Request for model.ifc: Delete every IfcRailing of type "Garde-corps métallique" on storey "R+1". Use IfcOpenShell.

First a look at what the model holds.

```python
import ifcopenshell
import ifcopenshell.util.element

model = ifcopenshell.open("model.ifc")
print(model.schema)
storey = next(s for s in model.by_type("IfcBuildingStorey") if s.Name == "R+1")
railings = [e for e in ifcopenshell.util.element.get_decomposition(storey) if e.is_a("IfcRailing")]
seen = {}
for e in railings:
    element_type = ifcopenshell.util.element.get_type(e)
    name = element_type.Name if element_type not in (None, e) else None
    seen[name] = seen.get(name, 0) + 1
for name, count in sorted(seen.items(), key=str):
    print(count, "x", name)
```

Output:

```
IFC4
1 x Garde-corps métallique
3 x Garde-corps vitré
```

```python
import ifcopenshell
import ifcopenshell.api.root
import ifcopenshell.util.element

model = ifcopenshell.open("model.ifc")

storey = next(s for s in model.by_type("IfcBuildingStorey") if s.Name == "R+1")
railings = [e for e in ifcopenshell.util.element.get_decomposition(storey) if e.is_a("IfcRailing")]
targets = [e for e in railings if (t := ifcopenshell.util.element.get_type(e)) not in (None, e) and t.Name == "Garde-corps métallique"]

for e in targets:
    ifcopenshell.api.root.remove_product(model, product=e)
print(len(targets), "removed")

model.write("model-out.ifc")
```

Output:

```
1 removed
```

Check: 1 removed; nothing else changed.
